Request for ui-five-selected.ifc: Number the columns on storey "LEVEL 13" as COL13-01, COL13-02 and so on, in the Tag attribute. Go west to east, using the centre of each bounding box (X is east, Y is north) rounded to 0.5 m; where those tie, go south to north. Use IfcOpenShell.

First a look at what the model holds.

```python
import ifcopenshell
import ifcopenshell.util.element
import ifcopenshell.util.placement

model = ifcopenshell.open("ui-five-selected.ifc")
print(model.schema)
storey = next(s for s in model.by_type("IfcBuildingStorey") if s.Name == "LEVEL 13")
columns = [e for e in ifcopenshell.util.element.get_decomposition(storey) if e.is_a("IfcColumn")]
for e in sorted(columns, key=lambda e: e.id()):
    origin = ifcopenshell.util.placement.get_local_placement(e.ObjectPlacement)[:3, 3]
    print(e.id(), e.Tag, e.Name, origin.round(2) + 0.0, sep=" | ")
```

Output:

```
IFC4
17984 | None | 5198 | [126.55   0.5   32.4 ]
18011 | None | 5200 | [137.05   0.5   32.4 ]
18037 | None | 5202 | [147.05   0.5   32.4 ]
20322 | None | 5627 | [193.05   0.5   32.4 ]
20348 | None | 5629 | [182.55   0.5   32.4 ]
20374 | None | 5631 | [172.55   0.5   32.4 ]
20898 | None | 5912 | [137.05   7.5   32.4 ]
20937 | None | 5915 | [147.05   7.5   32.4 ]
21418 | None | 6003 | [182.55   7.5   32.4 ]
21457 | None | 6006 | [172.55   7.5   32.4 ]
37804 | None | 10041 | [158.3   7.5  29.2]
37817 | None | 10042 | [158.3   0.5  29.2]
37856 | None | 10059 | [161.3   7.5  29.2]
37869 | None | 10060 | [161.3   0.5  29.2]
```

```python
import ifcopenshell
import ifcopenshell.geom
import ifcopenshell.util.element
import ifcopenshell.util.shape

model = ifcopenshell.open("ui-five-selected.ifc")
settings = ifcopenshell.geom.settings()
settings.set("use-world-coords", True)


def centre(element):
    shape = ifcopenshell.geom.create_shape(settings, element)
    return ifcopenshell.util.shape.get_bbox_centroid(shape.geometry)


storey = next(s for s in model.by_type("IfcBuildingStorey") if s.Name == "LEVEL 13")
columns = [e for e in ifcopenshell.util.element.get_decomposition(storey) if e.is_a("IfcColumn")]

# Insertion points can sit at a corner or the storey origin, so sort by the geometry (in metres).
centres = {e: centre(e) for e in columns}
columns.sort(key=lambda e: (round(centres[e][0] / 0.5), centres[e][1]))

for i, e in enumerate(columns, start=1):
    number = f"COL13-{i:02d}"
    e.Tag = number
    print(e.id(), number)

model.write("ui-five-selected_edited.ifc")
```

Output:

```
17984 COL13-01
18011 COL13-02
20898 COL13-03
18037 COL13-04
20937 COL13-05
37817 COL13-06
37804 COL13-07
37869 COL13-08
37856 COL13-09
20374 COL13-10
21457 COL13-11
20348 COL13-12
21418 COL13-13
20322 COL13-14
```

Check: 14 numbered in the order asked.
